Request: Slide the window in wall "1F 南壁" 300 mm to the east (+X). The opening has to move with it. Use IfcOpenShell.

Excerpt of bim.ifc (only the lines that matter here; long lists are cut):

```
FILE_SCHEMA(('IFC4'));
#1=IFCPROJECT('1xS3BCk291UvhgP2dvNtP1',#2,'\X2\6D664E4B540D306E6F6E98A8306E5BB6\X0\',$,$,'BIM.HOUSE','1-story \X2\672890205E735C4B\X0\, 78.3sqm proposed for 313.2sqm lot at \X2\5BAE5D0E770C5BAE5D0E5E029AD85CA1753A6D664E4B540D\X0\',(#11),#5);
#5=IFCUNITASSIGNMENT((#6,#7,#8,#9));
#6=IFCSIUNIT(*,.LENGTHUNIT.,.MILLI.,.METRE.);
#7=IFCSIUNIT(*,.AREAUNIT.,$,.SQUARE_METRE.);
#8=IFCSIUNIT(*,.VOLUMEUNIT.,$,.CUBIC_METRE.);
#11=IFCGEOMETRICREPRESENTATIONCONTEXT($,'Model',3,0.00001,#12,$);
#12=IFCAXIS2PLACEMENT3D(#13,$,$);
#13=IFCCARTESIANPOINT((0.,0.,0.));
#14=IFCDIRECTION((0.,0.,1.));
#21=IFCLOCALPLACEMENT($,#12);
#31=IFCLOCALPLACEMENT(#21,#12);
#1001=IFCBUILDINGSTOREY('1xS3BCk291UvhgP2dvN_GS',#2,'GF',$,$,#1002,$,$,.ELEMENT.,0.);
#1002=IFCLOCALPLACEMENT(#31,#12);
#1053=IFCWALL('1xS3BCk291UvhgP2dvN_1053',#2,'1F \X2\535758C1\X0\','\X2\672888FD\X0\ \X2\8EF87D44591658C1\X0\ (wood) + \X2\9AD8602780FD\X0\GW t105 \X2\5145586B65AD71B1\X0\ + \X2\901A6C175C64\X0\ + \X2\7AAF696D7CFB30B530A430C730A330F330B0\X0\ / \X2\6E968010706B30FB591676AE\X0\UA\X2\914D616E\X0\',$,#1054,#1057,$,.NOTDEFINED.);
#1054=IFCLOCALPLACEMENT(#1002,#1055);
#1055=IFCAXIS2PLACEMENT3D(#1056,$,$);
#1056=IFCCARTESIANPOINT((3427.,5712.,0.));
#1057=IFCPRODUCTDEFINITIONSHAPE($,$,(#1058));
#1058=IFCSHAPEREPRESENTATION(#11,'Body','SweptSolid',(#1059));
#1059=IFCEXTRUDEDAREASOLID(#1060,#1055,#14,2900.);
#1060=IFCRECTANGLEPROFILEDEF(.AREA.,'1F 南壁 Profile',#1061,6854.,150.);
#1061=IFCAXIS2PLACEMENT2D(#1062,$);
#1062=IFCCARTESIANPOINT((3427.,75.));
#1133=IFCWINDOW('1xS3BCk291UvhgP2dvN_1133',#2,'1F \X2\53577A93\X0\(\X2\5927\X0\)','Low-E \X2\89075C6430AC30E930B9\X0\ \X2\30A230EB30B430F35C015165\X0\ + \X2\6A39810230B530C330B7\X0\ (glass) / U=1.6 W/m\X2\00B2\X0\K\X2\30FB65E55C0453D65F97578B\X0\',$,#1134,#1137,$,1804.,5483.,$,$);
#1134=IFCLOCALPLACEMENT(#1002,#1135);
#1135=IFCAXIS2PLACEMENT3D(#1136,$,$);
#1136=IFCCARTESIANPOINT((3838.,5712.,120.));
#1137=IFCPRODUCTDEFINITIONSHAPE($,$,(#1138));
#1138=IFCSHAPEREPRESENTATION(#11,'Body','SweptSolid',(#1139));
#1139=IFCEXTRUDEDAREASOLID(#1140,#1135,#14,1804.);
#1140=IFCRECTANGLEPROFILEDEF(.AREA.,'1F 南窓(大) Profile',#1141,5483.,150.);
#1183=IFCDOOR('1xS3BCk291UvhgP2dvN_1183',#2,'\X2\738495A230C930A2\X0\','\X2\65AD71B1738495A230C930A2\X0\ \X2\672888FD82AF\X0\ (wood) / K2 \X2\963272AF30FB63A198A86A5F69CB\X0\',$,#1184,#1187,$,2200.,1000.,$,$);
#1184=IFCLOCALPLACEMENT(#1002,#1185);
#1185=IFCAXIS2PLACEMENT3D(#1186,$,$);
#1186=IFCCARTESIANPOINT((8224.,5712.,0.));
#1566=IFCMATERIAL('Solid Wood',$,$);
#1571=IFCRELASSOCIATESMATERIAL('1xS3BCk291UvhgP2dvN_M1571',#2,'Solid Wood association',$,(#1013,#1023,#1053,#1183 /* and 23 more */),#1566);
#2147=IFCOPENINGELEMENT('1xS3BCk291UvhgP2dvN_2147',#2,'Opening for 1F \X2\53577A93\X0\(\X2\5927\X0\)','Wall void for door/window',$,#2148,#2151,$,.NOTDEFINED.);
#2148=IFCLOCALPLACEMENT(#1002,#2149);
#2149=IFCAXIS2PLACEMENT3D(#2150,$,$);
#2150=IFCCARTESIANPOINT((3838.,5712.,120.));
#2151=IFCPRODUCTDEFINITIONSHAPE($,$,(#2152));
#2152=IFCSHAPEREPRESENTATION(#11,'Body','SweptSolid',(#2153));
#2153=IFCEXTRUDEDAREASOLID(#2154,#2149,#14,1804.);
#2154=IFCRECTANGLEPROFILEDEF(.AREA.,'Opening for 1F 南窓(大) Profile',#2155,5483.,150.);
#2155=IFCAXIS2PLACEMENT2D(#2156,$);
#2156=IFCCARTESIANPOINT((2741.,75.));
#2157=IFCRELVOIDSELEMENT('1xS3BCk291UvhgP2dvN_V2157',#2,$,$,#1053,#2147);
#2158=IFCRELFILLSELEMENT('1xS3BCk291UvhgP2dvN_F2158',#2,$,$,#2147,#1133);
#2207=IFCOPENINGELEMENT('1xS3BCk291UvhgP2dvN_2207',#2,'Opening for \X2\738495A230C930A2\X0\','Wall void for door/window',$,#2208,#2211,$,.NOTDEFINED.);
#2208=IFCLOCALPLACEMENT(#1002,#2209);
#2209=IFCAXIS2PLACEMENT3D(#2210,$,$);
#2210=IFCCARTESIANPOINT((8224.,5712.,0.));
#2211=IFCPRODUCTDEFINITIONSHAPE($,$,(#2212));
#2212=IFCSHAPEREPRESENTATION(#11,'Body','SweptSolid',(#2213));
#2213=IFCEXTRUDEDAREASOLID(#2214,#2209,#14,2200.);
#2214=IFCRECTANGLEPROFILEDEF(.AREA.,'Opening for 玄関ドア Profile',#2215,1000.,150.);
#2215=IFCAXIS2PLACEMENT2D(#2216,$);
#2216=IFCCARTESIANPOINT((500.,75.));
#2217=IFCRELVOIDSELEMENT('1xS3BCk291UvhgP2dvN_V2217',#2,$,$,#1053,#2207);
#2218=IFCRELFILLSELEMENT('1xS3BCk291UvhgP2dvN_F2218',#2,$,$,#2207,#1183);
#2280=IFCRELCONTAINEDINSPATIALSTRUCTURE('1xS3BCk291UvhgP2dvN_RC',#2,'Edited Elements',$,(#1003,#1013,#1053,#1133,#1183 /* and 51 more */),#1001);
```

```python
import ifcopenshell
import ifcopenshell.api.geometry
import ifcopenshell.util.placement

model = ifcopenshell.open("bim.ifc")

window = model.by_guid("1xS3BCk291UvhgP2dvN_1133")
opening = window.FillsVoids[0].RelatingOpeningElement
wall = opening.VoidsElements[0].RelatingBuildingElement

wall_matrix = ifcopenshell.util.placement.get_local_placement(wall.ObjectPlacement)
shift = wall_matrix[:3, 0] * 300.0
before = ifcopenshell.util.placement.get_local_placement(window.ObjectPlacement)[:3, 3].copy()

# The window is not placed relative to its opening, so move both.
for product in (opening, window):
    matrix = ifcopenshell.util.placement.get_local_placement(product.ObjectPlacement)
    matrix[:3, 3] += shift
    ifcopenshell.api.geometry.edit_object_placement(model, product=product, matrix=matrix, is_si=False)

after = ifcopenshell.util.placement.get_local_placement(window.ObjectPlacement)[:3, 3]
print("window moved by", (after - before).round(3) + 0.0)

model.write("bim_edited.ifc")
```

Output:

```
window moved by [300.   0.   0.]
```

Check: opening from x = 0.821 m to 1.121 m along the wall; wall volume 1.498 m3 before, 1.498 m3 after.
